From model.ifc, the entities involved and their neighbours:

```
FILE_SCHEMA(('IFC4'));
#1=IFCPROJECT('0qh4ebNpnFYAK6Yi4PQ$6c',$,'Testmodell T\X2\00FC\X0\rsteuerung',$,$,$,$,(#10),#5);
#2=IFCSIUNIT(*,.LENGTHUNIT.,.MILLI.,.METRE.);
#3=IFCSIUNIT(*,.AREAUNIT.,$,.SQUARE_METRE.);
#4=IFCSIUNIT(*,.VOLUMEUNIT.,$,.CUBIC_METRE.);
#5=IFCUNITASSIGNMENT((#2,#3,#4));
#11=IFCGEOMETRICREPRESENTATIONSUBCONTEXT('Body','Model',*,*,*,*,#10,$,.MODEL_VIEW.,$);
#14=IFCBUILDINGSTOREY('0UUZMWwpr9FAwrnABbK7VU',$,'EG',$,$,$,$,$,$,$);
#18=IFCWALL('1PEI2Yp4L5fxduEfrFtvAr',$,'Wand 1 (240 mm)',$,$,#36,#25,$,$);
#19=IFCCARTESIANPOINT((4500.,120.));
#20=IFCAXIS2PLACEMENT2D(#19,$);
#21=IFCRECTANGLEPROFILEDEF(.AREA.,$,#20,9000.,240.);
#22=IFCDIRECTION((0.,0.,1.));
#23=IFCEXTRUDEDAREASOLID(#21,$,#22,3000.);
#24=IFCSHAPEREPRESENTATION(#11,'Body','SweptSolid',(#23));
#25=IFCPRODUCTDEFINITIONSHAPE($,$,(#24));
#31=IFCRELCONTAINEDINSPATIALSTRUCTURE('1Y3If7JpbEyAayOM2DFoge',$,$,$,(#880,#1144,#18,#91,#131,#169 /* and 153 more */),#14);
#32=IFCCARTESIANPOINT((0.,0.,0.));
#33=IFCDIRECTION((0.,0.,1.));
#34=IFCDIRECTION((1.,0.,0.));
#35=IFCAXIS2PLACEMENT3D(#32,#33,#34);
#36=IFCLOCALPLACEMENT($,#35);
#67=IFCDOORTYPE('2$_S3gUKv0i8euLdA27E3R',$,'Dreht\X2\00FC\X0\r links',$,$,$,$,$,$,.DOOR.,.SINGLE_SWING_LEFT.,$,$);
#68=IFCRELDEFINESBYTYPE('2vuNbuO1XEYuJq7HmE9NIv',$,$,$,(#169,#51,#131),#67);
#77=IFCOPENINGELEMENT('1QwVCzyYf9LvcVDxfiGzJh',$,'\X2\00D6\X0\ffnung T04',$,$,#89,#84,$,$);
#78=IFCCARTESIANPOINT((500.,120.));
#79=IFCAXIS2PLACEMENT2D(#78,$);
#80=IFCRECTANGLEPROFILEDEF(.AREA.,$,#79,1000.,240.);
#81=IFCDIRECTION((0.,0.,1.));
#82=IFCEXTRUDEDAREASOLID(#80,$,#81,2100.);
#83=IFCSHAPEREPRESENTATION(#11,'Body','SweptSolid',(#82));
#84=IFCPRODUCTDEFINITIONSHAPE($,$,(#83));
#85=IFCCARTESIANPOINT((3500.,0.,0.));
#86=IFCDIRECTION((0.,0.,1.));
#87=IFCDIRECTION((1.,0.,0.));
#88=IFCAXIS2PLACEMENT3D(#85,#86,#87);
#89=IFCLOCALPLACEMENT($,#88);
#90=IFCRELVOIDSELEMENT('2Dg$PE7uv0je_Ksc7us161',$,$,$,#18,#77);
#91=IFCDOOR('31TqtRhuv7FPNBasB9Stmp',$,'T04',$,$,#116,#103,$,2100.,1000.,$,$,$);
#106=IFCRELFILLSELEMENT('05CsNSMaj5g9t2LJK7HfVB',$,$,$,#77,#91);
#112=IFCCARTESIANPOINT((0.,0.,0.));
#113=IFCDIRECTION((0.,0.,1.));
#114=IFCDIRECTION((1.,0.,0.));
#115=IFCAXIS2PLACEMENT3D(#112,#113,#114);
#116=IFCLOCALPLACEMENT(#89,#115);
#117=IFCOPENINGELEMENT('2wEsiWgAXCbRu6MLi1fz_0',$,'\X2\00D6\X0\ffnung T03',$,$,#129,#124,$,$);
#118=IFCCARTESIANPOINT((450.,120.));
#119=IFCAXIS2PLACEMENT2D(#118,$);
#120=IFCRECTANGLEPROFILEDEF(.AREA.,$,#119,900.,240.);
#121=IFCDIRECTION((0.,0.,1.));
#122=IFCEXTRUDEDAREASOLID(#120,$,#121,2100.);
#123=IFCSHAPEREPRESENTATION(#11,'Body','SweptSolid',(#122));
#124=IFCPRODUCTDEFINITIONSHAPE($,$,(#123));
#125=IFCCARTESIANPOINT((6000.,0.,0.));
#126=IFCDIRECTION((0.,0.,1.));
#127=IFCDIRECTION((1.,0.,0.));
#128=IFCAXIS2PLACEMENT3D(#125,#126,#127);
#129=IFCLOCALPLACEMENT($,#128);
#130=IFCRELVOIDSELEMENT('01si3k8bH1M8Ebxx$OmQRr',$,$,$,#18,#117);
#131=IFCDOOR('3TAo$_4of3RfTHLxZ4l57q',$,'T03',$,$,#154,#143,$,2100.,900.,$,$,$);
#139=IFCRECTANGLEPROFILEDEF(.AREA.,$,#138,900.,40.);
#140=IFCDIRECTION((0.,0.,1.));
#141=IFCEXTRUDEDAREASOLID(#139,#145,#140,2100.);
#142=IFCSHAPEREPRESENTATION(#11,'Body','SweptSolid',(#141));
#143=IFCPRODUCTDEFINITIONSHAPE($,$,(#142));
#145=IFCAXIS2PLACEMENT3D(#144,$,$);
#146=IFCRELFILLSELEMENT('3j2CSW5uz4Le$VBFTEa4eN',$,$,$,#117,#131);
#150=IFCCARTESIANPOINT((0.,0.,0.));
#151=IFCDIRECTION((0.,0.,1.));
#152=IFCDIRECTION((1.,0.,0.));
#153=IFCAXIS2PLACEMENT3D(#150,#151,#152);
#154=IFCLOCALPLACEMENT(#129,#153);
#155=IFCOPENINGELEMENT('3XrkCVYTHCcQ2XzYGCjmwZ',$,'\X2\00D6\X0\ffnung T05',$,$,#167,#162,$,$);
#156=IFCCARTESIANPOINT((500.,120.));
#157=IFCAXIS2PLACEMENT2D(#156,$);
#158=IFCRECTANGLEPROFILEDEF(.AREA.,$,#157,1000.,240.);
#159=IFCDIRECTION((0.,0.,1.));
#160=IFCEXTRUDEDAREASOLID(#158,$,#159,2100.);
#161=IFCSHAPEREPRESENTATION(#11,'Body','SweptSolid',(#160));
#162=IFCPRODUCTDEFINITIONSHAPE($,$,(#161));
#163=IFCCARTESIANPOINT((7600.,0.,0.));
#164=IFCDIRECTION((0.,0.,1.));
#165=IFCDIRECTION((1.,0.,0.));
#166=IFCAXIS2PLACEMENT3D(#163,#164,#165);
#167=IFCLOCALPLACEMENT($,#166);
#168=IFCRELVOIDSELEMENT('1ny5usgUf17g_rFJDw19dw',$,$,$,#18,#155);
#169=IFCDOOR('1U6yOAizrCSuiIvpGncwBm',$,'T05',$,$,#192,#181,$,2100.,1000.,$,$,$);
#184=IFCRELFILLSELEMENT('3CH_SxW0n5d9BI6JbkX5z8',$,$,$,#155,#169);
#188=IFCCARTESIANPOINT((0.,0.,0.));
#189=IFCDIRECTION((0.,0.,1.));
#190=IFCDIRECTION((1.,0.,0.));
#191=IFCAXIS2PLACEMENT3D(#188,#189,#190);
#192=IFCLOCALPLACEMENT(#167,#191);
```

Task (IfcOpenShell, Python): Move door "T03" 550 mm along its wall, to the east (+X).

```python
import ifcopenshell
import ifcopenshell.api.geometry
import ifcopenshell.util.placement

model = ifcopenshell.open("model.ifc")

door = model.by_guid("3TAo$_4of3RfTHLxZ4l57q")
opening = door.FillsVoids[0].RelatingOpeningElement
wall = opening.VoidsElements[0].RelatingBuildingElement

wall_matrix = ifcopenshell.util.placement.get_local_placement(wall.ObjectPlacement)
shift = wall_matrix[:3, 0] * 550.0
before = ifcopenshell.util.placement.get_local_placement(door.ObjectPlacement)[:3, 3].copy()

# The door is placed relative to its opening, so it follows when the opening moves.
matrix = ifcopenshell.util.placement.get_local_placement(opening.ObjectPlacement)
matrix[:3, 3] += shift
ifcopenshell.api.geometry.edit_object_placement(
    model, product=opening, matrix=matrix, is_si=False, should_transform_children=True
)

after = ifcopenshell.util.placement.get_local_placement(door.ObjectPlacement)[:3, 3]
print("door moved by", (after - before).round(3) + 0.0)

model.write("model_edited.ifc")
```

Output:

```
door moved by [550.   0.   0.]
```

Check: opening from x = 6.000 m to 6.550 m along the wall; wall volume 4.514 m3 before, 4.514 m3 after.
